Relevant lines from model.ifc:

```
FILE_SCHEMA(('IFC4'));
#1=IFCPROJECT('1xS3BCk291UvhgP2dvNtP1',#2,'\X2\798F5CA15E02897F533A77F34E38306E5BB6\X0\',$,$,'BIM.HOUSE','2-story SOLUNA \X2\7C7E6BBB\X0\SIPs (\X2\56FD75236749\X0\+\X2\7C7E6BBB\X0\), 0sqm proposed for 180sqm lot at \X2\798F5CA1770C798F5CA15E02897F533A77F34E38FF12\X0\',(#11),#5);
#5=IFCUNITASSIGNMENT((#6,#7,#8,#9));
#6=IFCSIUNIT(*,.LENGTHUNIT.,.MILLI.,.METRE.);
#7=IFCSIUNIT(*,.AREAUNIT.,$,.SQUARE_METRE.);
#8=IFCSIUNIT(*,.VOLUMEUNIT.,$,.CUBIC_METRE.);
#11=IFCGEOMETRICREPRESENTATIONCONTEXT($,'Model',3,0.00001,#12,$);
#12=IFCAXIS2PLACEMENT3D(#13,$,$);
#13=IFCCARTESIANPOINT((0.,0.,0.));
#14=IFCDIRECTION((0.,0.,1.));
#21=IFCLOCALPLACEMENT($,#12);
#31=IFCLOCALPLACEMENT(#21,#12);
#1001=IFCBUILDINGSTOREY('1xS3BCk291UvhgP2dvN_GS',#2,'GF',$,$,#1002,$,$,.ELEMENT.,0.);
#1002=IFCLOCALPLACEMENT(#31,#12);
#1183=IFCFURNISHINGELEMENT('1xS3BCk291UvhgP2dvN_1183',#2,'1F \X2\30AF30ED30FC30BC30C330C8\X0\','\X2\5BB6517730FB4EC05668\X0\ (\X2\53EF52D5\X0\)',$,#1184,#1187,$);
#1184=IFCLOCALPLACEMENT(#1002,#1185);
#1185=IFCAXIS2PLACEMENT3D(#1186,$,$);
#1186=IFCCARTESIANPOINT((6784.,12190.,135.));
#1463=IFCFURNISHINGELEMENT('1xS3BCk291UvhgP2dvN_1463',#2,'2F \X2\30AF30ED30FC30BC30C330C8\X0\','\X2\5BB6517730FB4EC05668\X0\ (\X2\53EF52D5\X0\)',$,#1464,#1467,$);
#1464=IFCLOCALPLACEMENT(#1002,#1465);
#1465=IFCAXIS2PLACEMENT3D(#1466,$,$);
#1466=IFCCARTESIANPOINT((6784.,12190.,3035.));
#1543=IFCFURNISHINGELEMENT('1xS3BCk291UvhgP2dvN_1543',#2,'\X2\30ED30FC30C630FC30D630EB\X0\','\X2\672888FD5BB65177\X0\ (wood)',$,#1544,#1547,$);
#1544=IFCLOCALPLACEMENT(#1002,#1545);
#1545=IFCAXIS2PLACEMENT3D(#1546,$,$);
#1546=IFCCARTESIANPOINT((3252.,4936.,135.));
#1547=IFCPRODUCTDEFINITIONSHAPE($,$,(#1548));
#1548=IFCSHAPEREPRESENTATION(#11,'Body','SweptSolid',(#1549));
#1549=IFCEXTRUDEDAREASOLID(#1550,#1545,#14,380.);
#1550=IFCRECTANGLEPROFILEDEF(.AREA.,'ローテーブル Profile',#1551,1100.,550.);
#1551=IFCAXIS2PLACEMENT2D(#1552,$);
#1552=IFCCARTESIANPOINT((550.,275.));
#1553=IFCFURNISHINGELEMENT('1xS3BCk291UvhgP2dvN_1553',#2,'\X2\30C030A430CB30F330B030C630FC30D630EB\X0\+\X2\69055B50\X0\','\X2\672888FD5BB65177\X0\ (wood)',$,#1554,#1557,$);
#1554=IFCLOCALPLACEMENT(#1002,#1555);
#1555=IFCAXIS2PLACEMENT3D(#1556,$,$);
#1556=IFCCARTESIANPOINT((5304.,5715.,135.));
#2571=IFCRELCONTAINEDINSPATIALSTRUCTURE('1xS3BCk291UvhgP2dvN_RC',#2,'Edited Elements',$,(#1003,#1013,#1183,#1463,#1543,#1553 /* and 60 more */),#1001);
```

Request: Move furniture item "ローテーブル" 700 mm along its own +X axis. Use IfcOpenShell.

```python
import ifcopenshell
import ifcopenshell.api.geometry
import ifcopenshell.util.placement

model = ifcopenshell.open("model.ifc")

item = model.by_id(1543)
matrix = ifcopenshell.util.placement.get_local_placement(item.ObjectPlacement)
matrix[:3, 3] += matrix[:3, 0] * 700.0
ifcopenshell.api.geometry.edit_object_placement(model, product=item, matrix=matrix, is_si=False)

print(ifcopenshell.util.placement.get_local_placement(item.ObjectPlacement).round(3) + 0.0)

model.write("model_v2.ifc")
```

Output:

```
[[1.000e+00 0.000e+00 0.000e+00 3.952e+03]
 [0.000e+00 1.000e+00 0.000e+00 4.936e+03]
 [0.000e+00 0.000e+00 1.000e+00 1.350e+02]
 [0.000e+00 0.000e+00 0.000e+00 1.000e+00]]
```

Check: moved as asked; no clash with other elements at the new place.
